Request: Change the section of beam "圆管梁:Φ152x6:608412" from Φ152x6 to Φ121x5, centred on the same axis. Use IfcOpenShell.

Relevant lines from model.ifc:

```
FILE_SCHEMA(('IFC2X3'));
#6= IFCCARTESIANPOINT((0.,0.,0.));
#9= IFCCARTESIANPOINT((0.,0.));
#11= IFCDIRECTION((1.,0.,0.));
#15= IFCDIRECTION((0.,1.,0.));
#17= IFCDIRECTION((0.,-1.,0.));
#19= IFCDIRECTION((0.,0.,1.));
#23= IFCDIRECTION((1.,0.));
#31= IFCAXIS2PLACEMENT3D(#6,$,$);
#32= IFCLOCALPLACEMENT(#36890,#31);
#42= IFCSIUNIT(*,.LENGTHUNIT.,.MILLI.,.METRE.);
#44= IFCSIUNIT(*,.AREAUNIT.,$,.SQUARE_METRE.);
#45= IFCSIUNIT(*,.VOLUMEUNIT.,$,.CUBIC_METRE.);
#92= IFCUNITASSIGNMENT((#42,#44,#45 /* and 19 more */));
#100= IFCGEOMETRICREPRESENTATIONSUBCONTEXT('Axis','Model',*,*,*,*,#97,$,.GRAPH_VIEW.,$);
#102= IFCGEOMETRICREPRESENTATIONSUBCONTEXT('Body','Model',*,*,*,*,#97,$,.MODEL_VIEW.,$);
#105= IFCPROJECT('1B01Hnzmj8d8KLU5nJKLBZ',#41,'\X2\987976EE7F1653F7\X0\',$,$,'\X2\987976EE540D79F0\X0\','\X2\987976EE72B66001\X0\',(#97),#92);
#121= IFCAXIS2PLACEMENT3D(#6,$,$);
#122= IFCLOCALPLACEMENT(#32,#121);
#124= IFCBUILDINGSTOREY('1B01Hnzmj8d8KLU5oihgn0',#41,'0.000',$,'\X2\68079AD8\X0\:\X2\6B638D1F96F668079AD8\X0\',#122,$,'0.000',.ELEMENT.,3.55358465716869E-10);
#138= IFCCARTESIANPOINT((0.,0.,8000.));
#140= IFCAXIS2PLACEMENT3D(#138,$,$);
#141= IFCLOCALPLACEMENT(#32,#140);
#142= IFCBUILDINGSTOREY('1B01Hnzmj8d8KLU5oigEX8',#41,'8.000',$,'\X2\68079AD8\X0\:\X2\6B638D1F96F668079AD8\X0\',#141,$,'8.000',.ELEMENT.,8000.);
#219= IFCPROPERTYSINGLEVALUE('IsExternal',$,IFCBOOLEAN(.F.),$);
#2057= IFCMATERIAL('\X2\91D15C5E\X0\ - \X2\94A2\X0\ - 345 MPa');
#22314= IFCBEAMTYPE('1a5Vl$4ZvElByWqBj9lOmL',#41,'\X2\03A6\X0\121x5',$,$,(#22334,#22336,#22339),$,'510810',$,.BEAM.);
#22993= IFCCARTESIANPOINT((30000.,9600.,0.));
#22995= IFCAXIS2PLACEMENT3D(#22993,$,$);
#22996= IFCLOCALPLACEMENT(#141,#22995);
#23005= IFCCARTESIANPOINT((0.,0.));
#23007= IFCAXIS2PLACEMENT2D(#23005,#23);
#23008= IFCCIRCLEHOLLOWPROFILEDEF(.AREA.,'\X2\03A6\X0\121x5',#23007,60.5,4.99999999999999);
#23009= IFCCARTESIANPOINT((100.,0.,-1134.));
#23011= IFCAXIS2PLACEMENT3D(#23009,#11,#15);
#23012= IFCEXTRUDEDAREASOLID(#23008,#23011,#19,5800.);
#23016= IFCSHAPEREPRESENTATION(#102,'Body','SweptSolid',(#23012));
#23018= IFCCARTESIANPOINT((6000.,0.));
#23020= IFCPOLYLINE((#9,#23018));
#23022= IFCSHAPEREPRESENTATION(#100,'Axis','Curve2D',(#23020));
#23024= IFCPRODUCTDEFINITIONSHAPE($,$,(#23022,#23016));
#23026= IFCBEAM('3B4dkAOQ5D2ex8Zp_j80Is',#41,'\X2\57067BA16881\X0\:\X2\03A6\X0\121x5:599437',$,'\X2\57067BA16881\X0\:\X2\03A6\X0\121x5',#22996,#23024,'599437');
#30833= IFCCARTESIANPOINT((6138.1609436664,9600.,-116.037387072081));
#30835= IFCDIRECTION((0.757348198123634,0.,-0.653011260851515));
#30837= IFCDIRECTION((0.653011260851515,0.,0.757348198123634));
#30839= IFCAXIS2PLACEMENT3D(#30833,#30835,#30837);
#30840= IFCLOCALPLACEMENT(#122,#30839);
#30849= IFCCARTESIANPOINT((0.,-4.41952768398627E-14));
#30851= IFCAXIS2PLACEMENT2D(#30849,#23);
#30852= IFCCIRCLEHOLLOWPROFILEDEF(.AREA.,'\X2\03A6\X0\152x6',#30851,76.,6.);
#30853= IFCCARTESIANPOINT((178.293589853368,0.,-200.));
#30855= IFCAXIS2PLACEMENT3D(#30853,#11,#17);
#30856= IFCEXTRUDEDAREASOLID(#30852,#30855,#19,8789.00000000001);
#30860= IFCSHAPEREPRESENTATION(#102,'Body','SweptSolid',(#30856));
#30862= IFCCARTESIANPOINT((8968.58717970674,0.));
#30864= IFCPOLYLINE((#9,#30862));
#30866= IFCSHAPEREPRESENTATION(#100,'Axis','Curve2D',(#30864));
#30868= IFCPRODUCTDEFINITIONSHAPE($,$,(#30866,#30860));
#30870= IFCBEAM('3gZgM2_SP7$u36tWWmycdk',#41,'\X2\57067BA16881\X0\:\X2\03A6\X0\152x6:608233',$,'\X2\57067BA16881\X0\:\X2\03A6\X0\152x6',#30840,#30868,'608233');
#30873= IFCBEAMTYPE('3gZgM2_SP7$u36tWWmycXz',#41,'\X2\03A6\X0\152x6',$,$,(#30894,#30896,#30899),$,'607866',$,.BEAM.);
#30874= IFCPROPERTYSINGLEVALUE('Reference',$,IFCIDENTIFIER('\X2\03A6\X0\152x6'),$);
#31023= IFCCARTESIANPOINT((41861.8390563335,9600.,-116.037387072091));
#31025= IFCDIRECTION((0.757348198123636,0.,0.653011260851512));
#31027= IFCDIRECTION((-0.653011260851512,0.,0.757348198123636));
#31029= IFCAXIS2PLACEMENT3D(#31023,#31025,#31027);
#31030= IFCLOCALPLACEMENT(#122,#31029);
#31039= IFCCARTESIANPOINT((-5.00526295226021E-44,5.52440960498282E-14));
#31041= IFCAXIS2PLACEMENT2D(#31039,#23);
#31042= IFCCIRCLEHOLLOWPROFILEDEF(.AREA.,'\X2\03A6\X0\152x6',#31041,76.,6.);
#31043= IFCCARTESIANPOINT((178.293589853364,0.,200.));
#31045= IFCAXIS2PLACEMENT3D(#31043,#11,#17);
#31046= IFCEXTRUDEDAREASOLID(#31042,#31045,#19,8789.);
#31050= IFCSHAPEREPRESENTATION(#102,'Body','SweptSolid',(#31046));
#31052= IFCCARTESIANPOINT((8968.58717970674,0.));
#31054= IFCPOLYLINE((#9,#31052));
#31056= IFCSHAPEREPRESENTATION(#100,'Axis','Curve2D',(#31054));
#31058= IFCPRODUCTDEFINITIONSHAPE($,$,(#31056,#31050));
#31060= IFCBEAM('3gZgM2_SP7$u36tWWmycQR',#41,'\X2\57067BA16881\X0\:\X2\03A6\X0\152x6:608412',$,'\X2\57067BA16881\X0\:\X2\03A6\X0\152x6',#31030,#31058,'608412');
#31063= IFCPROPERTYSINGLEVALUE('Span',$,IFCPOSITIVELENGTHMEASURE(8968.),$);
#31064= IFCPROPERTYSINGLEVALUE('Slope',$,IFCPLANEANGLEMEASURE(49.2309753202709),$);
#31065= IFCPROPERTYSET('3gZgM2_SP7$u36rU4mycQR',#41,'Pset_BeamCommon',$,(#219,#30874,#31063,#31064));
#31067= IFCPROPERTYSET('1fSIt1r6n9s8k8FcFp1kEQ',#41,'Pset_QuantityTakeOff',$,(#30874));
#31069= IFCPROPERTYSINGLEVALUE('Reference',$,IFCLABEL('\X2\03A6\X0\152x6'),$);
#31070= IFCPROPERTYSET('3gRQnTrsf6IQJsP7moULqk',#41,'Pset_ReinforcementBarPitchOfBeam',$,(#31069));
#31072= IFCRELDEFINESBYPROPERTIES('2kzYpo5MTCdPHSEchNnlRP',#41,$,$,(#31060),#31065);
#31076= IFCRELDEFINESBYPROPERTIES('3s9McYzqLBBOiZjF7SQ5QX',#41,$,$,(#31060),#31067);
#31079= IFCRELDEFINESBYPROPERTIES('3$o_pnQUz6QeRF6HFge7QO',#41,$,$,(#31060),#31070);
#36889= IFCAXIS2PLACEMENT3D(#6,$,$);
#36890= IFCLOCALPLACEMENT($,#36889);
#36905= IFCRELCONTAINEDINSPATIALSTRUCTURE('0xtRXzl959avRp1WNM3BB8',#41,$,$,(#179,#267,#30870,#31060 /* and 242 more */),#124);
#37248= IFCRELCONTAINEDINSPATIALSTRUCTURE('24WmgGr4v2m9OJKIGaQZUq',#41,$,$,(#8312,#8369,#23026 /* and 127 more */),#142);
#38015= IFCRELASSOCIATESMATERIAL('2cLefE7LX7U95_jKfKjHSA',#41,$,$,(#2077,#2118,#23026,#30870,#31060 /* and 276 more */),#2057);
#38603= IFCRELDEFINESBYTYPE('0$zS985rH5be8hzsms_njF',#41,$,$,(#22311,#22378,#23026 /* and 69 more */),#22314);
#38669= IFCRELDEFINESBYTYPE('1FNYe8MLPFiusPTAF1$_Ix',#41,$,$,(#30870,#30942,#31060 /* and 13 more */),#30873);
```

```python
import ifcopenshell
import ifcopenshell.api.pset
import ifcopenshell.api.type
import ifcopenshell.util.element
import ifcopenshell.util.representation

model = ifcopenshell.open("model.ifc")

member = model.by_guid("3gZgM2_SP7$u36tWWmycQR")
source = next(p for p in model.by_type("IfcCircleHollowProfileDef") if p.ProfileName == "Φ121x5")

body = ifcopenshell.util.representation.get_representation(member, "Model", "Body")
solid = body.Items[0]
old_profile = solid.SweptArea

# Copy the section's sizes but keep this member's own profile position.
profile = ifcopenshell.util.element.copy(model, source)
profile.Position = old_profile.Position
solid.SweptArea = profile
if not model.get_total_inverses(old_profile):
    ifcopenshell.util.element.remove_deep2(model, old_profile)

new_type = model.by_guid("1a5Vl$4ZvElByWqBj9lOmL")
ifcopenshell.api.type.assign_type(
    model, related_objects=[member], relating_type=new_type, should_map_representations=False
)
member.Name = member.Name.replace("Φ152x6", "Φ121x5")
member.ObjectType = "圆管梁:Φ121x5"
pset = model.by_id(ifcopenshell.util.element.get_pset(member, "Pset_BeamCommon", should_inherit=False)["id"])
ifcopenshell.api.pset.edit_pset(model, pset=pset, properties={"Reference": "Φ121x5"})
pset = model.by_id(ifcopenshell.util.element.get_pset(member, "Pset_QuantityTakeOff", should_inherit=False)["id"])
ifcopenshell.api.pset.edit_pset(model, pset=pset, properties={"Reference": "Φ121x5"})
pset = model.by_id(ifcopenshell.util.element.get_pset(member, "Pset_ReinforcementBarPitchOfBeam", should_inherit=False)["id"])
ifcopenshell.api.pset.edit_pset(model, pset=pset, properties={"Reference": "Φ121x5"})

print(solid.SweptArea)

model.write("model_edited.ifc")
```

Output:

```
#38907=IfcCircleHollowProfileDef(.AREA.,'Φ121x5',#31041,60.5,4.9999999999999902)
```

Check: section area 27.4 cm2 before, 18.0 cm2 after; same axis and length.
